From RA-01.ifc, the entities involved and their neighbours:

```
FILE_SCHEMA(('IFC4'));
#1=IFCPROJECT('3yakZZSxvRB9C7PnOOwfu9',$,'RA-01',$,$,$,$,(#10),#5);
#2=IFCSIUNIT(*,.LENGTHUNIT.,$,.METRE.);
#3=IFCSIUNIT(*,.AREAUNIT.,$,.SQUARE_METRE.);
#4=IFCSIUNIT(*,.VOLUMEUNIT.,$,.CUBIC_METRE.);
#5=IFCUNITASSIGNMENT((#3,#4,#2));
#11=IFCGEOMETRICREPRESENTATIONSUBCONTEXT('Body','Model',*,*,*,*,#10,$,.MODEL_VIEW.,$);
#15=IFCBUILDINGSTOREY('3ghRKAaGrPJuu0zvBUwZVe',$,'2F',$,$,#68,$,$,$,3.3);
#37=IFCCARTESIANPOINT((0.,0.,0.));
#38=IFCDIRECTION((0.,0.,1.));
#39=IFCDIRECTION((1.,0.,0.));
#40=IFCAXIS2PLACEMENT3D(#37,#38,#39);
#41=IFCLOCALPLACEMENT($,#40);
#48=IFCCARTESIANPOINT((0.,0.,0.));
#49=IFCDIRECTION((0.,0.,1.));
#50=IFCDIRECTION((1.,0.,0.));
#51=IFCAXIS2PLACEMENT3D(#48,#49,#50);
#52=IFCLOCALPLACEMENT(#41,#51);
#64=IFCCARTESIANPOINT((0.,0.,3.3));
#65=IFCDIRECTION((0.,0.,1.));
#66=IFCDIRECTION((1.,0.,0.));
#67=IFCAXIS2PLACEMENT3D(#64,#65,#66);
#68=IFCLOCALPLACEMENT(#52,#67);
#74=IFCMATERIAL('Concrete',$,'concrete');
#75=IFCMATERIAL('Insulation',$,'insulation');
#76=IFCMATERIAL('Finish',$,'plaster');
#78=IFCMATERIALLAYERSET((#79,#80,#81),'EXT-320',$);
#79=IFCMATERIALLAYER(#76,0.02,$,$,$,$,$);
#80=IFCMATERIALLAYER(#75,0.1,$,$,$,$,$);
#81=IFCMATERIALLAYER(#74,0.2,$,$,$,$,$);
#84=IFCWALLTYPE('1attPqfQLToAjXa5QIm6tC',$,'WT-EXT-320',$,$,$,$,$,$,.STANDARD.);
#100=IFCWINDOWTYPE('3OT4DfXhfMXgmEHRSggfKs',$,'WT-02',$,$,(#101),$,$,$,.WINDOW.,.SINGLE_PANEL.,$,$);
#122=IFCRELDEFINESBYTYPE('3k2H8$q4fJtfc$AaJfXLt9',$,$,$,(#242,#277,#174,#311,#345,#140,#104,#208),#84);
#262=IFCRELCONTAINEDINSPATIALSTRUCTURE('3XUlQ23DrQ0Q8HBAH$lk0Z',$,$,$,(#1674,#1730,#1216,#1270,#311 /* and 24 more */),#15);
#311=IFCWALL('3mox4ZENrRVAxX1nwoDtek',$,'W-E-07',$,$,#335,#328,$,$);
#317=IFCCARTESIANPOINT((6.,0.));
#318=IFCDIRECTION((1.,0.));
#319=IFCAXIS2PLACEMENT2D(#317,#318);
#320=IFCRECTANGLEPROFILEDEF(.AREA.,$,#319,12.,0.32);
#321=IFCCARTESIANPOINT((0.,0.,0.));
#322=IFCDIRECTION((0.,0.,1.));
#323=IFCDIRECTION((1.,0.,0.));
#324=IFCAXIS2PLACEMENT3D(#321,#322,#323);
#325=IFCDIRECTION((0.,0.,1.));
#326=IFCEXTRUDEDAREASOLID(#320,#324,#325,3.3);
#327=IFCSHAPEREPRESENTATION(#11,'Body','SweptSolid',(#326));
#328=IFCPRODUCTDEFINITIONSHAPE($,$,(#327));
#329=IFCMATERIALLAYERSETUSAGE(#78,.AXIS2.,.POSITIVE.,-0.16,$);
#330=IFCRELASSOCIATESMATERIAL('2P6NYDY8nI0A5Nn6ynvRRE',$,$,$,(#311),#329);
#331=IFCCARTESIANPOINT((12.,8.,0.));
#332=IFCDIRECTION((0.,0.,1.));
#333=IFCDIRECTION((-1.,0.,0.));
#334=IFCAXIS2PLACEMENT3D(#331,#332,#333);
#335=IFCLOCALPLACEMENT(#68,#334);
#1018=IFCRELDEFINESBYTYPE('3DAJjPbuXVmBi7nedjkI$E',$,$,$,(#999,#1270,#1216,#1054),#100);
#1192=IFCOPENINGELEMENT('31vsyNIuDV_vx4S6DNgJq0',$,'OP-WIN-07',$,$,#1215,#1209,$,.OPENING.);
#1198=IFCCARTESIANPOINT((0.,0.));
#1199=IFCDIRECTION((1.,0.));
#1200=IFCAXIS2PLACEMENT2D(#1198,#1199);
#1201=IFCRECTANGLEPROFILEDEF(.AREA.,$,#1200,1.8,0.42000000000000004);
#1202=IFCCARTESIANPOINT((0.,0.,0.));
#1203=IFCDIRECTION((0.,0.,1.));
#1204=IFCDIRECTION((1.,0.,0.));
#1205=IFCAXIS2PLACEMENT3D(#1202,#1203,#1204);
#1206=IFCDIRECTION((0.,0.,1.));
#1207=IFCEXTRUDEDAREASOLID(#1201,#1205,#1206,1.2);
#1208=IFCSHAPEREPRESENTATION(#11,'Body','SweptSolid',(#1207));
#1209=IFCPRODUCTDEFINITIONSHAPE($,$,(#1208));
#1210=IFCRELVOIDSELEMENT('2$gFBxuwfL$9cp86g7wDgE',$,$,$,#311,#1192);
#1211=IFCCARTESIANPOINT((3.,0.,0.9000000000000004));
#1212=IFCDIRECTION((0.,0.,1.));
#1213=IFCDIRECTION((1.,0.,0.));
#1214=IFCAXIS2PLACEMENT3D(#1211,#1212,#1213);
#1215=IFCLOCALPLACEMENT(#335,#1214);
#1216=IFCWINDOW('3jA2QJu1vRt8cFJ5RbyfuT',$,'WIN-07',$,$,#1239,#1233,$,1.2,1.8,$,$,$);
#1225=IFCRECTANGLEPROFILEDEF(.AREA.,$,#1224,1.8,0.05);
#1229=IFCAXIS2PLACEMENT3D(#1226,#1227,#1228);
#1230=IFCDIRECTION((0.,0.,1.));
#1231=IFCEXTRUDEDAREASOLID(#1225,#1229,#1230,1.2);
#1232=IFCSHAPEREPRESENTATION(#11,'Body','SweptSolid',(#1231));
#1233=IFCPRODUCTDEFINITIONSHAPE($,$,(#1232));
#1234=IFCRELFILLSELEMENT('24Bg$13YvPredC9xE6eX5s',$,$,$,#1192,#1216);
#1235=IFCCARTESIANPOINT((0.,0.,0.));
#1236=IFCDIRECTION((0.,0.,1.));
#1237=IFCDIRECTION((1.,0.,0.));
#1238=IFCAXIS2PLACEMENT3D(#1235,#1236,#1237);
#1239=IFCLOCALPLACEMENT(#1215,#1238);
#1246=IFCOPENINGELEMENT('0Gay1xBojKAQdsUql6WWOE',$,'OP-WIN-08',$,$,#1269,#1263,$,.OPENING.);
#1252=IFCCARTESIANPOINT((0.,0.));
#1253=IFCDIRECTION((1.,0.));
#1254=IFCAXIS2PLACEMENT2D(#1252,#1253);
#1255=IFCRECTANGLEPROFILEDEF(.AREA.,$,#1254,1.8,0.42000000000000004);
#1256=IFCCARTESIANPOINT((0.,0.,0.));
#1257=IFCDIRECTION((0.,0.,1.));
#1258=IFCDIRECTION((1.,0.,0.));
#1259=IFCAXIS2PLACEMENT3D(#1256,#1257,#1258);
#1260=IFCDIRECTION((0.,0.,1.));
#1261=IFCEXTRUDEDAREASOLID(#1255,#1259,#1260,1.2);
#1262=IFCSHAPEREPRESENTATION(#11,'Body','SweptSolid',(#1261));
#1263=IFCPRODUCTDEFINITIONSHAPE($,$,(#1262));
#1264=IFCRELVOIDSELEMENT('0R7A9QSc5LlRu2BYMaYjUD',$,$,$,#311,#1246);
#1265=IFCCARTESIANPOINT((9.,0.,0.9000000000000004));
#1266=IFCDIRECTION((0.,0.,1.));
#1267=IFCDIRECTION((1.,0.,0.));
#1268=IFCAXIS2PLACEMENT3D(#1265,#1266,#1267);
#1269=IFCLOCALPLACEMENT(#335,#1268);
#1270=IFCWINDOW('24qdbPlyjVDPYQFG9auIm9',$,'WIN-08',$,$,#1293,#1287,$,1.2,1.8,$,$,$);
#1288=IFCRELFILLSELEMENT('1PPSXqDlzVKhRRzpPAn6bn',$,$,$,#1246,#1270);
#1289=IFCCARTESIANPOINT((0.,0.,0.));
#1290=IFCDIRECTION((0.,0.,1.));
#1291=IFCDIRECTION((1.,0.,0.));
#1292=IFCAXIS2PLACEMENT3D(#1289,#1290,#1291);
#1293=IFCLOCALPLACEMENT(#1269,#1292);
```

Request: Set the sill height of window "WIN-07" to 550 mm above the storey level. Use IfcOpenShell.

```python
import numpy as np
import ifcopenshell
import ifcopenshell.api.geometry
import ifcopenshell.geom
import ifcopenshell.util.element
import ifcopenshell.util.placement
import ifcopenshell.util.shape
import ifcopenshell.util.unit

model = ifcopenshell.open("RA-01.ifc")
unit_scale = ifcopenshell.util.unit.calculate_unit_scale(model)

window = model.by_id(1216)
opening = window.FillsVoids[0].RelatingOpeningElement
storey = ifcopenshell.util.element.get_container(window, ifc_class="IfcBuildingStorey")
level = ifcopenshell.util.placement.get_local_placement(storey.ObjectPlacement)[2, 3]

# The opening's origin need not be at the sill, so measure its lowest point.
shape = ifcopenshell.geom.create_shape(ifcopenshell.geom.settings(), opening)
bottom = ifcopenshell.util.shape.get_shape_bottom_elevation(shape, shape.geometry) / unit_scale
dz = level + 0.55 / unit_scale - bottom

shift = np.array([0.0, 0.0, dz])
# The window is placed relative to its opening, so it follows when the opening moves.
matrix = ifcopenshell.util.placement.get_local_placement(opening.ObjectPlacement)
matrix[:3, 3] += shift
ifcopenshell.api.geometry.edit_object_placement(
    model, product=opening, matrix=matrix, is_si=False, should_transform_children=True
)

print(f"moved by {dz * unit_scale:+.3f} m")

model.write("RA-01_updated.ifc")
```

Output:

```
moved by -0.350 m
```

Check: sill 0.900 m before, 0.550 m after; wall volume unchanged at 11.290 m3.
